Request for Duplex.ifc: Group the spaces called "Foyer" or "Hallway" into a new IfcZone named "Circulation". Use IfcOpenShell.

First a look at what the model holds.

```python
import ifcopenshell

model = ifcopenshell.open("Duplex.ifc")
print(model.schema)
seen = {}
for space in model.by_type("IfcSpace"):
    seen[space.LongName] = seen.get(space.LongName, 0) + 1
for name, count in sorted(seen.items(), key=str):
    print(count, "x", name)
print("zones:", [z.Name for z in model.by_type("IfcZone")][:20])
```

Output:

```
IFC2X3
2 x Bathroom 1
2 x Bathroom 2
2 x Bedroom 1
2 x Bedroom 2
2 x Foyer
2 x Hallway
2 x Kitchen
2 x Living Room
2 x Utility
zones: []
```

```python
import ifcopenshell
import ifcopenshell.api.group
import ifcopenshell.api.root

model = ifcopenshell.open("Duplex.ifc")

names = {"Foyer", "Hallway"}
spaces = [s for s in model.by_type("IfcSpace") if s.LongName in names]

zone = ifcopenshell.api.root.create_entity(model, ifc_class="IfcZone", name="Circulation")
ifcopenshell.api.group.assign_group(model, products=spaces, group=zone)
print(len(spaces), "spaces in", zone.Name)

model.write("Duplex_rev.ifc")
```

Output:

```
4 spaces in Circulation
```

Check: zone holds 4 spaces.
